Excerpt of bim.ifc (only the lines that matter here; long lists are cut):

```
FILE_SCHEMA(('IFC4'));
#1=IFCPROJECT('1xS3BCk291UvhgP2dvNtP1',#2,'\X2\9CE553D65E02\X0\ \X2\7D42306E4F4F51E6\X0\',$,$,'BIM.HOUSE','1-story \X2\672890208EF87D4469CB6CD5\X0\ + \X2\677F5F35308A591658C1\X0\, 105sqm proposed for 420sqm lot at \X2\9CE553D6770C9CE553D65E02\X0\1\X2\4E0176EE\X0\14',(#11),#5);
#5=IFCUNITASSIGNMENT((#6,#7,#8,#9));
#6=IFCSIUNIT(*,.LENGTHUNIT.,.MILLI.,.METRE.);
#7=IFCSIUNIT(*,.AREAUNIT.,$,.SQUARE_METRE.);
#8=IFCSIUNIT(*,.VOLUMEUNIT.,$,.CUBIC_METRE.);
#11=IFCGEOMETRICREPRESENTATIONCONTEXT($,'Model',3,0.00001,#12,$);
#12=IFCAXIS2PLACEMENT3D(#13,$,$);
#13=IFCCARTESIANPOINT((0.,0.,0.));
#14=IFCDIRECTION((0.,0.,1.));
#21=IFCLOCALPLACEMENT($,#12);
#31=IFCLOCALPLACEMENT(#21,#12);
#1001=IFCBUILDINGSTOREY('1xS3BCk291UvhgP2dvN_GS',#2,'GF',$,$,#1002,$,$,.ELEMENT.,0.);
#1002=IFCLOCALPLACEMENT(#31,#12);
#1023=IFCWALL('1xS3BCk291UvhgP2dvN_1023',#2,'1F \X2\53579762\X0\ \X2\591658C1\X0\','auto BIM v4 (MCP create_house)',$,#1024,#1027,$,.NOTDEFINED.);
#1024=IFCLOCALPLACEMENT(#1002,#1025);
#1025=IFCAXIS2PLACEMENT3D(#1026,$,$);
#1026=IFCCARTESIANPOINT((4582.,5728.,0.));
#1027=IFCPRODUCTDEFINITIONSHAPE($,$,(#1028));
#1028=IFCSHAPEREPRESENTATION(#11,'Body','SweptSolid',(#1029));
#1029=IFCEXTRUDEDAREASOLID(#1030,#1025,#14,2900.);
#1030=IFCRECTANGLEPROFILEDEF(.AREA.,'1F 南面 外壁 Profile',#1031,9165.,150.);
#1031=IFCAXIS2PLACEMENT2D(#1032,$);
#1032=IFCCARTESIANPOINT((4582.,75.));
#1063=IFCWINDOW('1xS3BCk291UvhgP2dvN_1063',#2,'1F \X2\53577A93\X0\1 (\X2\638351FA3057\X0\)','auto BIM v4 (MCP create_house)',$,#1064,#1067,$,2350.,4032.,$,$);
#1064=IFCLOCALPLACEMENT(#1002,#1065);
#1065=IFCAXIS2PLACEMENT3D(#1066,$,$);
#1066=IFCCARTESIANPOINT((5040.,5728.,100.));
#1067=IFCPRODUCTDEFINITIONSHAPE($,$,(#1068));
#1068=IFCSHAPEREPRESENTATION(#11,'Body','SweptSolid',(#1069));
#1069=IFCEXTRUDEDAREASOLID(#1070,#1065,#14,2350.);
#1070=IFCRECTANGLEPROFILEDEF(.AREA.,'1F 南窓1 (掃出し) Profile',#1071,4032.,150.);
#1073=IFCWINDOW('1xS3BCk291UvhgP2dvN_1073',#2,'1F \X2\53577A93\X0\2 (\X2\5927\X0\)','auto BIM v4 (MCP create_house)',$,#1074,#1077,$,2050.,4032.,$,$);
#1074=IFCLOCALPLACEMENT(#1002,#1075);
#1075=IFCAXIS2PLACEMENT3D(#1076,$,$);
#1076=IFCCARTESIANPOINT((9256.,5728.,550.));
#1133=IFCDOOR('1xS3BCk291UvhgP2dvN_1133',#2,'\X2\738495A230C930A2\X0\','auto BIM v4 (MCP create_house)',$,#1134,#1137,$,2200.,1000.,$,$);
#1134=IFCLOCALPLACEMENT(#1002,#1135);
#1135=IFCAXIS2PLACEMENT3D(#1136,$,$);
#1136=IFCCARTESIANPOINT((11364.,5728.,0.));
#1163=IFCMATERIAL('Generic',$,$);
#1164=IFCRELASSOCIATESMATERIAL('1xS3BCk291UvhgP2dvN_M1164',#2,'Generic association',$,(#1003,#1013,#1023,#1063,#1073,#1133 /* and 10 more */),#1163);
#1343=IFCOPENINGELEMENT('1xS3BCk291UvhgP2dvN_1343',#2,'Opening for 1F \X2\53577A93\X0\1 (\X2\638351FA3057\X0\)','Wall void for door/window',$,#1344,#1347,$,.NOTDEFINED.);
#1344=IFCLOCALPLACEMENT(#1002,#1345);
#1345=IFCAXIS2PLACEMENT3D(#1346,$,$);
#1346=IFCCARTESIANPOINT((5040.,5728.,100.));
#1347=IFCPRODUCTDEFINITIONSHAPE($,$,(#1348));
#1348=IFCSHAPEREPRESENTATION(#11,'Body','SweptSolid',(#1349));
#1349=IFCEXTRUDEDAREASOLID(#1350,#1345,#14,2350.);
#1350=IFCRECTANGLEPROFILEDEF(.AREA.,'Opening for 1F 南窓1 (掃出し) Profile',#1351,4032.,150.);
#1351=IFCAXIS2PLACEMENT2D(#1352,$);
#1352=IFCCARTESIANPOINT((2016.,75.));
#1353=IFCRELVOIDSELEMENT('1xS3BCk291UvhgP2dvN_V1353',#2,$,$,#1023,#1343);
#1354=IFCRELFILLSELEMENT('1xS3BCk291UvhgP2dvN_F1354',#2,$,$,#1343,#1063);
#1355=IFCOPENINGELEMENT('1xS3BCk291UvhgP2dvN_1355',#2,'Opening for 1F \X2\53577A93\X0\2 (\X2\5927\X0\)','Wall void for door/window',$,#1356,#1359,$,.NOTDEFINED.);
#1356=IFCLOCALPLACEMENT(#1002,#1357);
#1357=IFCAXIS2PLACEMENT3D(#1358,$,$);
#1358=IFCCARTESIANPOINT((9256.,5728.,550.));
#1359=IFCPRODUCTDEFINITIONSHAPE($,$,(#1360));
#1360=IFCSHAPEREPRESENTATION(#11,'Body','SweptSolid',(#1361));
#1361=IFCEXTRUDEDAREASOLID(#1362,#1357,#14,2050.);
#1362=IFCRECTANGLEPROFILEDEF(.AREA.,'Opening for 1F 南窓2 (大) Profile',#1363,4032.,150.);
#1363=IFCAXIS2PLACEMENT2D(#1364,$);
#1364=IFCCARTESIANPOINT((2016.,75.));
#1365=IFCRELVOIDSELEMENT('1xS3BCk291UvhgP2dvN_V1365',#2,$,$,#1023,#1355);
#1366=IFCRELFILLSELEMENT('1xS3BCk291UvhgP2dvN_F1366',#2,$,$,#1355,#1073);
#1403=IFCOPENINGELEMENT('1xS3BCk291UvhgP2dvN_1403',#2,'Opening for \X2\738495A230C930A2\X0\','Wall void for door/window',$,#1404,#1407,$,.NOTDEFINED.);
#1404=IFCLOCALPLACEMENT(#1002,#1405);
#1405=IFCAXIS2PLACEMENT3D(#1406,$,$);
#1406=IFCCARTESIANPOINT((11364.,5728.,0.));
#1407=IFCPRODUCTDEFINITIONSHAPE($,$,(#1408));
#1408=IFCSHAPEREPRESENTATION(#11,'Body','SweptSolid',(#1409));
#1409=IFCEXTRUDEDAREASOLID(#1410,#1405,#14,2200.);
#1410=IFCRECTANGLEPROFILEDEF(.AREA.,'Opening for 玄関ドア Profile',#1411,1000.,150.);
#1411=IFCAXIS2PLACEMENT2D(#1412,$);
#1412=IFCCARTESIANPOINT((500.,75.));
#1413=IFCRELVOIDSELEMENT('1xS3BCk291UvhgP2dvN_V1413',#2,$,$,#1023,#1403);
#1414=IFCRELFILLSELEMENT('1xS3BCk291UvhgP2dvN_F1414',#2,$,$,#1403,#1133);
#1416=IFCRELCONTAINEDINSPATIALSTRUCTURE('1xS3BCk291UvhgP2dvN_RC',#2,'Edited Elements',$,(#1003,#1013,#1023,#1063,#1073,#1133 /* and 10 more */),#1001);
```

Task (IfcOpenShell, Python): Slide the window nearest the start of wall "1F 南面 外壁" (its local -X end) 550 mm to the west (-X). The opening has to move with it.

```python
import ifcopenshell
import ifcopenshell.api.geometry
import ifcopenshell.util.placement
import ifcopenshell.util.unit

model = ifcopenshell.open("bim.ifc")
unit_scale = ifcopenshell.util.unit.calculate_unit_scale(model)

window = model.by_guid("1xS3BCk291UvhgP2dvN_1063")
opening = window.FillsVoids[0].RelatingOpeningElement
wall = opening.VoidsElements[0].RelatingBuildingElement

wall_matrix = ifcopenshell.util.placement.get_local_placement(wall.ObjectPlacement)
shift = wall_matrix[:3, 0] * -0.55 / unit_scale
before = ifcopenshell.util.placement.get_local_placement(window.ObjectPlacement)[:3, 3].copy()

# The window is not placed relative to its opening, so move both.
for product in (opening, window):
    matrix = ifcopenshell.util.placement.get_local_placement(product.ObjectPlacement)
    matrix[:3, 3] += shift
    ifcopenshell.api.geometry.edit_object_placement(model, product=product, matrix=matrix, is_si=False)

after = ifcopenshell.util.placement.get_local_placement(window.ObjectPlacement)[:3, 3]
print("window moved by", (after - before).round(3) + 0.0)

model.write("bim_updated.ifc")
```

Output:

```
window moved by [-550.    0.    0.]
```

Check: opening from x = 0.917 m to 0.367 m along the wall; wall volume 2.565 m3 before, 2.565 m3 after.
